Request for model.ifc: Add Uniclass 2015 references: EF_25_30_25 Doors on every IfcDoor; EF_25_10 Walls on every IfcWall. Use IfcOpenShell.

First a look at what the model holds.

```python
import ifcopenshell

model = ifcopenshell.open("model.ifc")
print(model.schema)
print("classifications:", [c.Name for c in model.by_type("IfcClassification")])
for ifc_class in ("IfcDoor", "IfcRoof", "IfcStair", "IfcWall", "IfcWindow"):
    print(ifc_class, len(model.by_type(ifc_class)))
```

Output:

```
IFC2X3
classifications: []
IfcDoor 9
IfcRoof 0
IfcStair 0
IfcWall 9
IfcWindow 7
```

```python
import ifcopenshell
import ifcopenshell.api.classification

model = ifcopenshell.open("model.ifc")

# IFC2X3 requires Source and Edition and has no link from the project to the system.
system = model.create_entity("IfcClassification", Source="NBS", Edition="2015", Name="Uniclass 2015")

codes = {
    "IfcDoor": ("EF_25_30_25", "Doors"),
    "IfcWall": ("EF_25_10", "Walls"),
}
for ifc_class, (code, name) in codes.items():
    products = model.by_type(ifc_class)
    ifcopenshell.api.classification.add_reference(
        model, products=products, classification=system, identification=code, name=name
    )
    print(code, len(products))

model.write("model_updated.ifc")
```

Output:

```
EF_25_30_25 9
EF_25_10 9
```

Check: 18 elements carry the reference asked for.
